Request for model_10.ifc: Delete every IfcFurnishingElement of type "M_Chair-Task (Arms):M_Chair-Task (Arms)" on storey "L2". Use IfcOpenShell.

First a look at what the model holds.

```python
import ifcopenshell
import ifcopenshell.util.element

model = ifcopenshell.open("model_10.ifc")
print(model.schema)
storey = next(s for s in model.by_type("IfcBuildingStorey") if s.Name == "L2")
furniture = [e for e in ifcopenshell.util.element.get_decomposition(storey) if e.is_a("IfcFurnishingElement")]
seen = {}
for e in furniture:
    element_type = ifcopenshell.util.element.get_type(e)
    name = element_type.Name if element_type not in (None, e) else None
    seen[name] = seen.get(name, 0) + 1
for name, count in sorted(seen.items(), key=str):
    print(count, "x", name)
```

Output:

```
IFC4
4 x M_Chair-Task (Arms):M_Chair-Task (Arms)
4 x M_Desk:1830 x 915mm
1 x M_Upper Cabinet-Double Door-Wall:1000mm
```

```python
import ifcopenshell
import ifcopenshell.api.root
import ifcopenshell.util.element

model = ifcopenshell.open("model_10.ifc")

storey = next(s for s in model.by_type("IfcBuildingStorey") if s.Name == "L2")
furniture = [e for e in ifcopenshell.util.element.get_decomposition(storey) if e.is_a("IfcFurnishingElement")]
targets = [e for e in furniture if (t := ifcopenshell.util.element.get_type(e)) not in (None, e) and t.Name == "M_Chair-Task (Arms):M_Chair-Task (Arms)"]

for e in targets:
    ifcopenshell.api.root.remove_product(model, product=e)
print(len(targets), "removed")

model.write("model_10_updated.ifc")
```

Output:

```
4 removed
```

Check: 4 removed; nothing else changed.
